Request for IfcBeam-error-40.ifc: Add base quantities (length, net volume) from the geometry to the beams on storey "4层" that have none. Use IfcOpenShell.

First a look at what the model holds.

```python
import ifcopenshell
import ifcopenshell.util.element
import ifcopenshell.util.unit

model = ifcopenshell.open("IfcBeam-error-40.ifc")
print(model.schema)
for unit_type in ("LENGTHUNIT", "AREAUNIT", "VOLUMEUNIT"):
    print(unit_type, ifcopenshell.util.unit.calculate_unit_scale(model, unit_type))
storey = next(s for s in model.by_type("IfcBuildingStorey") if s.Name == "4层")
beams = [e for e in ifcopenshell.util.element.get_decomposition(storey) if e.is_a("IfcBeam")]
for e in sorted(beams, key=lambda e: e.id()):
    print(e.id(), e.is_a(), e.Name, list(ifcopenshell.util.element.get_psets(e, qtos_only=True)), sep=" | ")
```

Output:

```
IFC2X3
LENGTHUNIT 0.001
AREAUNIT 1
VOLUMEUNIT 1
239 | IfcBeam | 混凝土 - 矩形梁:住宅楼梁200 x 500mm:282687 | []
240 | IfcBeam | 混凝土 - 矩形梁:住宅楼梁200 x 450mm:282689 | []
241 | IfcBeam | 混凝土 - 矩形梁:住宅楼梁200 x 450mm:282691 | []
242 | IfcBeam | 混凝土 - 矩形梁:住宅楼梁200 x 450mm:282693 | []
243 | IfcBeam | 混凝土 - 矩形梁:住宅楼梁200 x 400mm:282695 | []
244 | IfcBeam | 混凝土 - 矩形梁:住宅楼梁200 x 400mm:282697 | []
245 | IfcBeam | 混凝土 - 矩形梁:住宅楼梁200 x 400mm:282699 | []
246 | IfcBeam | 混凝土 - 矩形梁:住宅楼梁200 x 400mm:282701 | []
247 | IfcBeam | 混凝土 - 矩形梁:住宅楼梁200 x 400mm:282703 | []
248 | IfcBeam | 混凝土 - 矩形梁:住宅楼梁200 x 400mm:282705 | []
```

```python
import ifcopenshell
import ifcopenshell.api.pset
import ifcopenshell.geom
import ifcopenshell.util.element
import ifcopenshell.util.shape
import ifcopenshell.util.unit

model = ifcopenshell.open("IfcBeam-error-40.ifc")
unit_scale = ifcopenshell.util.unit.calculate_unit_scale(model)
volume_scale = ifcopenshell.util.unit.calculate_unit_scale(model, "VOLUMEUNIT")
settings = ifcopenshell.geom.settings()

storey = next(s for s in model.by_type("IfcBuildingStorey") if s.Name == "4层")
beams = [e for e in ifcopenshell.util.element.get_decomposition(storey) if e.is_a("IfcBeam")]

for e in sorted(beams, key=lambda e: e.id()):
    if ifcopenshell.util.element.get_psets(e, qtos_only=True, should_inherit=False):
        continue
    # Geometry comes back in metres, in the element's own axes.
    shape = ifcopenshell.geom.create_shape(settings, e)
    values = {
        "Length": ifcopenshell.util.shape.get_max_xyz(shape.geometry) / unit_scale,
        "NetVolume": ifcopenshell.util.shape.get_volume(shape.geometry) / volume_scale,
    }
    qto = ifcopenshell.api.pset.add_qto(model, product=e, name="BaseQuantities")
    ifcopenshell.api.pset.edit_qto(model, qto=qto, properties=values)
    print(e.id(), {k: round(v, 3) for k, v in values.items()})

model.write("IfcBeam-error-40_edited.ifc")
```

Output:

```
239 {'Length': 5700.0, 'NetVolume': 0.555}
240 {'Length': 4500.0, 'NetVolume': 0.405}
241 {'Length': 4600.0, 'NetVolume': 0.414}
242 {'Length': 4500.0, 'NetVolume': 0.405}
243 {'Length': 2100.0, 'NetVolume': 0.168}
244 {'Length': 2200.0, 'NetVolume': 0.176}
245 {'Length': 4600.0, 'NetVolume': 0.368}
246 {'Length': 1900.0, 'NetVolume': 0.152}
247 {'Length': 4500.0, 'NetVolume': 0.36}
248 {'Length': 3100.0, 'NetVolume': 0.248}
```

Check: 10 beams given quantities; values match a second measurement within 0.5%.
